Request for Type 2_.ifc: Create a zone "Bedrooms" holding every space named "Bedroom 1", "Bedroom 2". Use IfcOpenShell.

First a look at what the model holds.

```python
import ifcopenshell

model = ifcopenshell.open("Type 2_.ifc")
print(model.schema)
seen = {}
for space in model.by_type("IfcSpace"):
    seen[space.LongName] = seen.get(space.LongName, 0) + 1
for name, count in sorted(seen.items(), key=str):
    print(count, "x", name)
print("zones:", [z.Name for z in model.by_type("IfcZone")][:20])
```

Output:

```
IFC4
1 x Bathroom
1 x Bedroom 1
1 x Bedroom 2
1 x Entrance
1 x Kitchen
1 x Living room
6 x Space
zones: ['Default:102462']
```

```python
import ifcopenshell
import ifcopenshell.api.group
import ifcopenshell.api.root

model = ifcopenshell.open("Type 2_.ifc")

names = {"Bedroom 1", "Bedroom 2"}
spaces = [s for s in model.by_type("IfcSpace") if s.LongName in names]

zone = ifcopenshell.api.root.create_entity(model, ifc_class="IfcZone", name="Bedrooms")
ifcopenshell.api.group.assign_group(model, products=spaces, group=zone)
print(len(spaces), "spaces in", zone.Name)

model.write("Type 2__v2.ifc")
```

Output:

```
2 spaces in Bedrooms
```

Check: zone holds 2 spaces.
